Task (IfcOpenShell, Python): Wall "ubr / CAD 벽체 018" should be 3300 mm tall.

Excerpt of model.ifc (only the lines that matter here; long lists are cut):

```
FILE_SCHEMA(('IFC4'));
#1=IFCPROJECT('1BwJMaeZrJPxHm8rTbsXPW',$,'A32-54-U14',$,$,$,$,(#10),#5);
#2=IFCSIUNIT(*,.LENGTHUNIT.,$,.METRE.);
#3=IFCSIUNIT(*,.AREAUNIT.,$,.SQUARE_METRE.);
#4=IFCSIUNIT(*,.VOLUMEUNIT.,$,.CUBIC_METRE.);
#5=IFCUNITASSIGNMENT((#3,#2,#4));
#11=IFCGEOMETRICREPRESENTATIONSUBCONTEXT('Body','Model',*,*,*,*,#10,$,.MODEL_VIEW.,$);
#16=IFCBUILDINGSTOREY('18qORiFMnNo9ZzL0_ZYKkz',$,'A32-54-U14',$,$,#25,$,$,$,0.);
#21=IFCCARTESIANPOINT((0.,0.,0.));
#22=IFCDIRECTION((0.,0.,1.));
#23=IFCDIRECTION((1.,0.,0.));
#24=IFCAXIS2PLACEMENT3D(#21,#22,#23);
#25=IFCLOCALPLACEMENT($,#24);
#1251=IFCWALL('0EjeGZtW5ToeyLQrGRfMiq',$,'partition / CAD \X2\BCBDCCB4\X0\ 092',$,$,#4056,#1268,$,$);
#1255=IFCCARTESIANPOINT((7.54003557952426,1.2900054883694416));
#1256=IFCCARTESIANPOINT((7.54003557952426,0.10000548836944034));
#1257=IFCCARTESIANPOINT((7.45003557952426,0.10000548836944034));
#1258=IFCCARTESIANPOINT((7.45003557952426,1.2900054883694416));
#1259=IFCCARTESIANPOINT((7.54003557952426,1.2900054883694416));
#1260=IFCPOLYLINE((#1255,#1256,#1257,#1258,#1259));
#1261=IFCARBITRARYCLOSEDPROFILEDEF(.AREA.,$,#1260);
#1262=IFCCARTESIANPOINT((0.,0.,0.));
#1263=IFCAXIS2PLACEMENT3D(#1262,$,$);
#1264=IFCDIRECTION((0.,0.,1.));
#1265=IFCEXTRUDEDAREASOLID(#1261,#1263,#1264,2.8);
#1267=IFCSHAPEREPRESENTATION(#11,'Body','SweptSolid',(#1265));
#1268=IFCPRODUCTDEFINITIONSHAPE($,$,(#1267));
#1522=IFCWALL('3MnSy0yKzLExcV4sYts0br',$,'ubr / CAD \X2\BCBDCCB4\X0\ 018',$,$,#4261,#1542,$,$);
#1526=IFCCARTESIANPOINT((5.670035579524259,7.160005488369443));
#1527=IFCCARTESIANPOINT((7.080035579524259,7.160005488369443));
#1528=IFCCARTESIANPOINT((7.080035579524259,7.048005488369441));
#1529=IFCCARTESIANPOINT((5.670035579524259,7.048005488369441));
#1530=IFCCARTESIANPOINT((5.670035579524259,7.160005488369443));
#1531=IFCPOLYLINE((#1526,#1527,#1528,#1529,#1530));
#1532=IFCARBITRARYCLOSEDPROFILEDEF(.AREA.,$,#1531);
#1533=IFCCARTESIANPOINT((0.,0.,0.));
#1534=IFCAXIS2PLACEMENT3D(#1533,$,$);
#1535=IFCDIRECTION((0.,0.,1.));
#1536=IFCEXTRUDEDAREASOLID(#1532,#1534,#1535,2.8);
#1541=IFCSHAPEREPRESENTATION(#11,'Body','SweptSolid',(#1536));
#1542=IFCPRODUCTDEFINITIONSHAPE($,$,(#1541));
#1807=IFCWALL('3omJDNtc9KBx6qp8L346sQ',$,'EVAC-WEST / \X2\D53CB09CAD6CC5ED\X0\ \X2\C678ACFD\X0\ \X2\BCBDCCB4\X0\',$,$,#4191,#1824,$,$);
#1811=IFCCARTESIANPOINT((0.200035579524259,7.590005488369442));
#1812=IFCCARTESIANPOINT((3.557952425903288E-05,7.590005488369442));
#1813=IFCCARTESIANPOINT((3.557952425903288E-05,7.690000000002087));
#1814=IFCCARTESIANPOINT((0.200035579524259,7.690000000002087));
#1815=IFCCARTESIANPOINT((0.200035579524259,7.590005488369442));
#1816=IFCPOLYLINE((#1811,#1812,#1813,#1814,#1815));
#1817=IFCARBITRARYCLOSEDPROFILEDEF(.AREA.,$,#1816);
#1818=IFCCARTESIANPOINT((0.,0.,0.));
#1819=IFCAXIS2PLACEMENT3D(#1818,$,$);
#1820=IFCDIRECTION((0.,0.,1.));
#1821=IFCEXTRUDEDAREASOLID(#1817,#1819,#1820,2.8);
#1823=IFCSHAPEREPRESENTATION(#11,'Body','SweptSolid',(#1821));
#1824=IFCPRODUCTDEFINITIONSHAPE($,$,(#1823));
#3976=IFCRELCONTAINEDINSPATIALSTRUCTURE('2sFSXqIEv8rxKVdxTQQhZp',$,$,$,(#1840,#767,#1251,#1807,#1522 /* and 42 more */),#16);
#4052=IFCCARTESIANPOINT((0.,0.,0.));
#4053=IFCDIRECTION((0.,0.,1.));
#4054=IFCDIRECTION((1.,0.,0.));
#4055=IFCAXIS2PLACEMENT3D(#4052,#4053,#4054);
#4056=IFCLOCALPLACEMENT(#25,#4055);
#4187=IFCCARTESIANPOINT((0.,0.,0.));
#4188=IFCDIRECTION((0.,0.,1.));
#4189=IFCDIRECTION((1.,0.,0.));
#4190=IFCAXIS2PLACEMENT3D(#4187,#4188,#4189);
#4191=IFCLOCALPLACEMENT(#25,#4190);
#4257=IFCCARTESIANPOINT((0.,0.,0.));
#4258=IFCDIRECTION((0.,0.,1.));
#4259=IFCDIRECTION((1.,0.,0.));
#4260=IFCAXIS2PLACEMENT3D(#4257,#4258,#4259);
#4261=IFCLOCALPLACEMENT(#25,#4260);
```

```python
import ifcopenshell
import ifcopenshell.geom
import ifcopenshell.util.representation
import ifcopenshell.util.shape
import ifcopenshell.util.unit

model = ifcopenshell.open("model.ifc")
unit_scale = ifcopenshell.util.unit.calculate_unit_scale(model)
settings = ifcopenshell.geom.settings()


def volume(element):
    """Net volume in cubic metres, openings subtracted."""
    shape = ifcopenshell.geom.create_shape(settings, element)
    return ifcopenshell.util.shape.get_volume(shape.geometry)


wall = model.by_id(1522)
before = volume(wall)

body = ifcopenshell.util.representation.get_representation(wall, "Model", "Body")
solid = body.Items[0]
old_height = solid.Depth
solid.Depth = 3.3 / unit_scale
after = volume(wall)

print(f"height {old_height:g} -> {solid.Depth:g}, volume {before:.3f} -> {after:.3f} m3")

model.write("model_edited.ifc")
```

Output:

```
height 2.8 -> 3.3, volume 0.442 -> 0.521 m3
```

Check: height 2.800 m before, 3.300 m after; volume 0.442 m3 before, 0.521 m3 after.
